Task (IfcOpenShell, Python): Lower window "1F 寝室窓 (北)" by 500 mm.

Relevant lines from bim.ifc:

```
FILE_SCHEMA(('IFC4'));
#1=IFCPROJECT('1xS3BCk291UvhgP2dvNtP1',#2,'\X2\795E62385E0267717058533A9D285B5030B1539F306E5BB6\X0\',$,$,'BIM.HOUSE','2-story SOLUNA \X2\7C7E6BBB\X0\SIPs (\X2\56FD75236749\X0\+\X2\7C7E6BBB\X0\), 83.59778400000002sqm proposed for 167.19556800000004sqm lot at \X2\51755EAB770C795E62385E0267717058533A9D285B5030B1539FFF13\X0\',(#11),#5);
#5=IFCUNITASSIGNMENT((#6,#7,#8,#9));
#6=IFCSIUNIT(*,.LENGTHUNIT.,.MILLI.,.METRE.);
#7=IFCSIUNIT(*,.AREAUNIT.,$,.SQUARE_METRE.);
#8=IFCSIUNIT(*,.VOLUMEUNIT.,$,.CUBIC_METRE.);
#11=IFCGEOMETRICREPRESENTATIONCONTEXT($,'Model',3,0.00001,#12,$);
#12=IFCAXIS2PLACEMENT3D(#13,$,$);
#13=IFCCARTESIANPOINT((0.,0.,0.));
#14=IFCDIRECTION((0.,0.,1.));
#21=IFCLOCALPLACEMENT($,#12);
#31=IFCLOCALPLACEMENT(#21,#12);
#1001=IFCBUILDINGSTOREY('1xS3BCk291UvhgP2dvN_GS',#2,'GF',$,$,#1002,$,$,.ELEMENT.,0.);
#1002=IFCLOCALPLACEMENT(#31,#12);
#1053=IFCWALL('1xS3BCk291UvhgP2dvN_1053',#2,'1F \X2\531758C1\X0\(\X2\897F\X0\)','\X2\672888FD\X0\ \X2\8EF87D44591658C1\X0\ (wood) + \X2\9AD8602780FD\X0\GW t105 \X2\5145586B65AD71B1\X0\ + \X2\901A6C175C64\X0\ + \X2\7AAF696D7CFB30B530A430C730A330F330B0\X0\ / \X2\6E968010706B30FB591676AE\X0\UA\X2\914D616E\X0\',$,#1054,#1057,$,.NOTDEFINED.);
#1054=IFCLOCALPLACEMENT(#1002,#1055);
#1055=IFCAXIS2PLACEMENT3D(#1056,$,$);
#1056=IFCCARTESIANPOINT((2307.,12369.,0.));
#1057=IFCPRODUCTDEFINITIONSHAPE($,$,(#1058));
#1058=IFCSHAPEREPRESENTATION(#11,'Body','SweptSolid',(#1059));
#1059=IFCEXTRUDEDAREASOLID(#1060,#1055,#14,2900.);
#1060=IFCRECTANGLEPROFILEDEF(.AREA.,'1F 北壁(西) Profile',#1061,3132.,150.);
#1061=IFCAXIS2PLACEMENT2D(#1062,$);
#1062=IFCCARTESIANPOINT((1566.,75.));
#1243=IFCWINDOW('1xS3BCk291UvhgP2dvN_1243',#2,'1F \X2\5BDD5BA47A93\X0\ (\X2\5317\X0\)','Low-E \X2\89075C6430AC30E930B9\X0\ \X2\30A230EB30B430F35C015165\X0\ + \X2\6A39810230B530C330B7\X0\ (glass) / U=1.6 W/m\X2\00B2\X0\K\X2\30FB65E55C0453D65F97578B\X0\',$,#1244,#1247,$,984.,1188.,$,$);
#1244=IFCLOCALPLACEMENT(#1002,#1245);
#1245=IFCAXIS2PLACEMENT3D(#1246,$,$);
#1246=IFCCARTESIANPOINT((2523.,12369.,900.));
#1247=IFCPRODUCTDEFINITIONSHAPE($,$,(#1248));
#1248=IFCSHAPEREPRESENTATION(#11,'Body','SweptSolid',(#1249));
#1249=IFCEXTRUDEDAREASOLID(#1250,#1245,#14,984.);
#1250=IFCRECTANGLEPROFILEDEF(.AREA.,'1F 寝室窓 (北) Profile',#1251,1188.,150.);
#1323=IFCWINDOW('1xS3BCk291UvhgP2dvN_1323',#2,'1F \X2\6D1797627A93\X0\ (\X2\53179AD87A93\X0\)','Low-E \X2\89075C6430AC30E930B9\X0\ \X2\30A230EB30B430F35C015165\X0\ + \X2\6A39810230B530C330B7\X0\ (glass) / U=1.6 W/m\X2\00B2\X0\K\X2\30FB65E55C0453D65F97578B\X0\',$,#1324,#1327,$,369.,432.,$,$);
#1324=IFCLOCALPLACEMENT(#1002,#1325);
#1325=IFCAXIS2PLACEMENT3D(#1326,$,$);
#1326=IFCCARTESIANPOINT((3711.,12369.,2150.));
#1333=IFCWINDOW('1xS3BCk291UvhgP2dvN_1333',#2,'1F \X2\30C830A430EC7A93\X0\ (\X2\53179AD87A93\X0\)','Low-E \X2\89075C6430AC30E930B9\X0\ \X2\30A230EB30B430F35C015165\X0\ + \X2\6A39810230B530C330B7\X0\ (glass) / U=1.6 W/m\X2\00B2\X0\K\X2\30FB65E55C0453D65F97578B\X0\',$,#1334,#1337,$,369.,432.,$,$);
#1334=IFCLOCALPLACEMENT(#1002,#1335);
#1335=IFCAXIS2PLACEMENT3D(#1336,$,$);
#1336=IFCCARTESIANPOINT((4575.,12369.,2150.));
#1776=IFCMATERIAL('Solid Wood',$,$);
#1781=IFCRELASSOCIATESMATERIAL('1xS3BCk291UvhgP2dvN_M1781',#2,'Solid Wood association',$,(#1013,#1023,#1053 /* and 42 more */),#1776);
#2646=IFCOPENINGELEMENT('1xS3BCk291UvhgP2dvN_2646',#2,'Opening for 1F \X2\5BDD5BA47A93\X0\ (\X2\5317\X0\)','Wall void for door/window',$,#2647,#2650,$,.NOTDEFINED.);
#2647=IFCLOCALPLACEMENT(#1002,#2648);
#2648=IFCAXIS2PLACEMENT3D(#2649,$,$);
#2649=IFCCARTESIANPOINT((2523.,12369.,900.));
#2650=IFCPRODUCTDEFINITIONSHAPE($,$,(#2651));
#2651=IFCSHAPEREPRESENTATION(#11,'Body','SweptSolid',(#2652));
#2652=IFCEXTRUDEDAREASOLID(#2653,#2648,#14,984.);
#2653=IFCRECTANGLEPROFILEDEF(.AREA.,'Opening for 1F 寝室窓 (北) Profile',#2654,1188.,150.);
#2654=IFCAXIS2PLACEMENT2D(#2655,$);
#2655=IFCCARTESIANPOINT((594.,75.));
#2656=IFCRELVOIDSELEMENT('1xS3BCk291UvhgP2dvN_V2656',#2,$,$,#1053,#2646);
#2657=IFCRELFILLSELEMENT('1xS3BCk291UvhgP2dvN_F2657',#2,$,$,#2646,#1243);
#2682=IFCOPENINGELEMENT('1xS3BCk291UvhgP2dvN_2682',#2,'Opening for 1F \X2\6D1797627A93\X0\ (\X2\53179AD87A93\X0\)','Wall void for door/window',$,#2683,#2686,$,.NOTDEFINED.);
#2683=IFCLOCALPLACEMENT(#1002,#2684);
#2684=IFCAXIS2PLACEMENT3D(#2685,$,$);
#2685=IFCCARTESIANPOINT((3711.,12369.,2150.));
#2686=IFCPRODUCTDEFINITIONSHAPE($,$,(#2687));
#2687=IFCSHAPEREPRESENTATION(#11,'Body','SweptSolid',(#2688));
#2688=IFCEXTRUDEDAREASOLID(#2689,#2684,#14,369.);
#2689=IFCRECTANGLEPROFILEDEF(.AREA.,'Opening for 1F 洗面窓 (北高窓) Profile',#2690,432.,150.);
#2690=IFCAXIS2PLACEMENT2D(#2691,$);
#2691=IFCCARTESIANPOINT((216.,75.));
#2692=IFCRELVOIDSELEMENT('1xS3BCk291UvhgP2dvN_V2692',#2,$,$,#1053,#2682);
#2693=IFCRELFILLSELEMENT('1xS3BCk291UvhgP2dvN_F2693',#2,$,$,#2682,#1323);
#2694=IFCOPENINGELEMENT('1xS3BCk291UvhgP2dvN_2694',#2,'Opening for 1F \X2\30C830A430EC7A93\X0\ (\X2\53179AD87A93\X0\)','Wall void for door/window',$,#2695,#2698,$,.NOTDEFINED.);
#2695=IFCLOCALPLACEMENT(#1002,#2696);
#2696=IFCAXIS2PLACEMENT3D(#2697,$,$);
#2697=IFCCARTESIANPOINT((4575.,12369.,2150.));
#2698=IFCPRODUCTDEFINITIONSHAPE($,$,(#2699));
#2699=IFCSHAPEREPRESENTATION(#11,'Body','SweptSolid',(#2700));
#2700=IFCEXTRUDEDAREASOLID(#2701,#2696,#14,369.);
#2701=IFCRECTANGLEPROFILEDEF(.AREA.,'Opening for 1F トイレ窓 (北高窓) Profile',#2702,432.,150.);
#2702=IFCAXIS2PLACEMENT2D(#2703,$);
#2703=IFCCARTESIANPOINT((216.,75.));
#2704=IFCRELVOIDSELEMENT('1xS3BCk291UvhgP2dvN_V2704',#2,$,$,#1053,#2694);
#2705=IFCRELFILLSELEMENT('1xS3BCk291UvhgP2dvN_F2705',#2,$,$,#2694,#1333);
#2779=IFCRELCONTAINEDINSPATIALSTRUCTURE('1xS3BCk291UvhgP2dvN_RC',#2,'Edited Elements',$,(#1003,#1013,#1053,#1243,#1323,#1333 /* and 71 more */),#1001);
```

```python
import numpy as np
import ifcopenshell
import ifcopenshell.api.geometry
import ifcopenshell.util.placement
import ifcopenshell.util.unit

model = ifcopenshell.open("bim.ifc")
unit_scale = ifcopenshell.util.unit.calculate_unit_scale(model)

window = model.by_id(1243)
opening = window.FillsVoids[0].RelatingOpeningElement
dz = -500.0

shift = np.array([0.0, 0.0, dz])
# The window is not placed relative to its opening, so move both.
for product in (opening, window):
    matrix = ifcopenshell.util.placement.get_local_placement(product.ObjectPlacement)
    matrix[:3, 3] += shift
    ifcopenshell.api.geometry.edit_object_placement(model, product=product, matrix=matrix, is_si=False)

print(f"moved by {dz * unit_scale:+.3f} m")

model.write("bim_rev.ifc")
```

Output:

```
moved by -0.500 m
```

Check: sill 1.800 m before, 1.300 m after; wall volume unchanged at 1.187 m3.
